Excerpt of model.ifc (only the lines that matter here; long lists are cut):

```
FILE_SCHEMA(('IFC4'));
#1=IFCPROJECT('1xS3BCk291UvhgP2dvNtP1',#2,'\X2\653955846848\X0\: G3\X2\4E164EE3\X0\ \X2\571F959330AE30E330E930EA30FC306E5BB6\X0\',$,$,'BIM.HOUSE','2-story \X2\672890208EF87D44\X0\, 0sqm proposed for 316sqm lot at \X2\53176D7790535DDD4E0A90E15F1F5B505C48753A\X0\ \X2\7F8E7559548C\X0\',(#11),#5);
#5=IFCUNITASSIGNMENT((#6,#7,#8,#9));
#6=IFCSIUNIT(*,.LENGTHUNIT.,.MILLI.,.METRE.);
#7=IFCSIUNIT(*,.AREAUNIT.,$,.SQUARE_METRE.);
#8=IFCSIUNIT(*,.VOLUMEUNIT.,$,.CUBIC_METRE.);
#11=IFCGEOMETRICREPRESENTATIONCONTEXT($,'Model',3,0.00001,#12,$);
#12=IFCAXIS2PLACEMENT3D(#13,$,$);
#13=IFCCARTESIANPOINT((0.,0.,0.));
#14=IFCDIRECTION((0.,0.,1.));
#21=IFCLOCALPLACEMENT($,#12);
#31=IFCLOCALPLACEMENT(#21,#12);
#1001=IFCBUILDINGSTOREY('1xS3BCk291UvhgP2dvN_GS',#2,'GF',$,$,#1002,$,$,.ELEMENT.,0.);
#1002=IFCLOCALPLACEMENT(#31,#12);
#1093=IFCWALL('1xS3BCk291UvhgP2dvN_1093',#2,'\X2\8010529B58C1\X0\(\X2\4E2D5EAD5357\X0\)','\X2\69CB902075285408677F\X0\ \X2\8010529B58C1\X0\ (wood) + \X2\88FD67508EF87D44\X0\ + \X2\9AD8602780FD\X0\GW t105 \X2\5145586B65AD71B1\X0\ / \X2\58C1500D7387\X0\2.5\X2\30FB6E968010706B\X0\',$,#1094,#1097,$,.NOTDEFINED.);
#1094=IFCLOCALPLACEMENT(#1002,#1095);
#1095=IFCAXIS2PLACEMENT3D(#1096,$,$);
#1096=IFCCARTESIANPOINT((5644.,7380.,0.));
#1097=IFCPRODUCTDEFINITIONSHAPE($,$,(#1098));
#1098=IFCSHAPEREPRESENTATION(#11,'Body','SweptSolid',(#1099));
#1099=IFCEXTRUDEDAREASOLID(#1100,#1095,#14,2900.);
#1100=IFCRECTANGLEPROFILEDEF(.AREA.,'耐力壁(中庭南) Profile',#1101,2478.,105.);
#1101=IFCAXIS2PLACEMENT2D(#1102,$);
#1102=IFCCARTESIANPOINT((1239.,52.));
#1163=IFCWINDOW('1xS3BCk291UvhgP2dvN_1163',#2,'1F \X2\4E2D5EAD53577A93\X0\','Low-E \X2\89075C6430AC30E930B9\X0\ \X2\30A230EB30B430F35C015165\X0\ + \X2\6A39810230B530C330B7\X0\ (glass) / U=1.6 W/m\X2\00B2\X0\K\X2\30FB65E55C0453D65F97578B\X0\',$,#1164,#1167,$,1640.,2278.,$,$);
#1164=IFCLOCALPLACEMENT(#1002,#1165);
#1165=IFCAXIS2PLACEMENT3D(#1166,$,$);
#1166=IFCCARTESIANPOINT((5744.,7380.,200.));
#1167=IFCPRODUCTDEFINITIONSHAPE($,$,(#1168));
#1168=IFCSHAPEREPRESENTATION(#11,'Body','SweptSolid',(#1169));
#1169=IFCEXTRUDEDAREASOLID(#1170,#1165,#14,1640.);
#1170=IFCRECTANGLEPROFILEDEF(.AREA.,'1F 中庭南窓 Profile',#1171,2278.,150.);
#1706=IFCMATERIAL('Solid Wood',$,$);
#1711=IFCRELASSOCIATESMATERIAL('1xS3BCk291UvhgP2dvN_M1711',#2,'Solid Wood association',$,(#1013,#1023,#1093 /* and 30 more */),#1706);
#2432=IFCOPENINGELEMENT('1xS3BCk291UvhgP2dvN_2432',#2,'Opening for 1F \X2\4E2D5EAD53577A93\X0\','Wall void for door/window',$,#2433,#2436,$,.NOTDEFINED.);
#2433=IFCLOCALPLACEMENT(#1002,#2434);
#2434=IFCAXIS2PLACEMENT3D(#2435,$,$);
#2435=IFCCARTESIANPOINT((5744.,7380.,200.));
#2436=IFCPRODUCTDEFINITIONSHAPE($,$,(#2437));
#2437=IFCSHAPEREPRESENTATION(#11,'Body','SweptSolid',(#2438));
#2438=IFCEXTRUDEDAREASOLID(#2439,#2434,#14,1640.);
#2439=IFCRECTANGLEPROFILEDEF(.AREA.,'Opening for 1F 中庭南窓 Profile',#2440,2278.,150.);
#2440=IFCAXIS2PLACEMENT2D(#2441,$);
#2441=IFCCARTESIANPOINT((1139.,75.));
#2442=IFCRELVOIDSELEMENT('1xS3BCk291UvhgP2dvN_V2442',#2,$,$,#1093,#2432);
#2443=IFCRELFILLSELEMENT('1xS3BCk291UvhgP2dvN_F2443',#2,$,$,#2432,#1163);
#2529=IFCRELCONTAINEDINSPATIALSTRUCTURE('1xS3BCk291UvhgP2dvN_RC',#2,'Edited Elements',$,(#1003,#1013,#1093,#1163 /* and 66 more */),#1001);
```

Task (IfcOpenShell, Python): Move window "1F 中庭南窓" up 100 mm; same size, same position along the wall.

```python
import numpy as np
import ifcopenshell
import ifcopenshell.api.geometry
import ifcopenshell.util.placement
import ifcopenshell.util.unit

model = ifcopenshell.open("model.ifc")
unit_scale = ifcopenshell.util.unit.calculate_unit_scale(model)

window = model.by_guid("1xS3BCk291UvhgP2dvN_1163")
opening = window.FillsVoids[0].RelatingOpeningElement
dz = 100.0

shift = np.array([0.0, 0.0, dz])
# The window is not placed relative to its opening, so move both.
for product in (opening, window):
    matrix = ifcopenshell.util.placement.get_local_placement(product.ObjectPlacement)
    matrix[:3, 3] += shift
    ifcopenshell.api.geometry.edit_object_placement(model, product=product, matrix=matrix, is_si=False)

print(f"moved by {dz * unit_scale:+.3f} m")

model.write("model_rev.ifc")
```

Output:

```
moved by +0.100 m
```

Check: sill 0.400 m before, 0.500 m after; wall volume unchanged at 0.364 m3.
